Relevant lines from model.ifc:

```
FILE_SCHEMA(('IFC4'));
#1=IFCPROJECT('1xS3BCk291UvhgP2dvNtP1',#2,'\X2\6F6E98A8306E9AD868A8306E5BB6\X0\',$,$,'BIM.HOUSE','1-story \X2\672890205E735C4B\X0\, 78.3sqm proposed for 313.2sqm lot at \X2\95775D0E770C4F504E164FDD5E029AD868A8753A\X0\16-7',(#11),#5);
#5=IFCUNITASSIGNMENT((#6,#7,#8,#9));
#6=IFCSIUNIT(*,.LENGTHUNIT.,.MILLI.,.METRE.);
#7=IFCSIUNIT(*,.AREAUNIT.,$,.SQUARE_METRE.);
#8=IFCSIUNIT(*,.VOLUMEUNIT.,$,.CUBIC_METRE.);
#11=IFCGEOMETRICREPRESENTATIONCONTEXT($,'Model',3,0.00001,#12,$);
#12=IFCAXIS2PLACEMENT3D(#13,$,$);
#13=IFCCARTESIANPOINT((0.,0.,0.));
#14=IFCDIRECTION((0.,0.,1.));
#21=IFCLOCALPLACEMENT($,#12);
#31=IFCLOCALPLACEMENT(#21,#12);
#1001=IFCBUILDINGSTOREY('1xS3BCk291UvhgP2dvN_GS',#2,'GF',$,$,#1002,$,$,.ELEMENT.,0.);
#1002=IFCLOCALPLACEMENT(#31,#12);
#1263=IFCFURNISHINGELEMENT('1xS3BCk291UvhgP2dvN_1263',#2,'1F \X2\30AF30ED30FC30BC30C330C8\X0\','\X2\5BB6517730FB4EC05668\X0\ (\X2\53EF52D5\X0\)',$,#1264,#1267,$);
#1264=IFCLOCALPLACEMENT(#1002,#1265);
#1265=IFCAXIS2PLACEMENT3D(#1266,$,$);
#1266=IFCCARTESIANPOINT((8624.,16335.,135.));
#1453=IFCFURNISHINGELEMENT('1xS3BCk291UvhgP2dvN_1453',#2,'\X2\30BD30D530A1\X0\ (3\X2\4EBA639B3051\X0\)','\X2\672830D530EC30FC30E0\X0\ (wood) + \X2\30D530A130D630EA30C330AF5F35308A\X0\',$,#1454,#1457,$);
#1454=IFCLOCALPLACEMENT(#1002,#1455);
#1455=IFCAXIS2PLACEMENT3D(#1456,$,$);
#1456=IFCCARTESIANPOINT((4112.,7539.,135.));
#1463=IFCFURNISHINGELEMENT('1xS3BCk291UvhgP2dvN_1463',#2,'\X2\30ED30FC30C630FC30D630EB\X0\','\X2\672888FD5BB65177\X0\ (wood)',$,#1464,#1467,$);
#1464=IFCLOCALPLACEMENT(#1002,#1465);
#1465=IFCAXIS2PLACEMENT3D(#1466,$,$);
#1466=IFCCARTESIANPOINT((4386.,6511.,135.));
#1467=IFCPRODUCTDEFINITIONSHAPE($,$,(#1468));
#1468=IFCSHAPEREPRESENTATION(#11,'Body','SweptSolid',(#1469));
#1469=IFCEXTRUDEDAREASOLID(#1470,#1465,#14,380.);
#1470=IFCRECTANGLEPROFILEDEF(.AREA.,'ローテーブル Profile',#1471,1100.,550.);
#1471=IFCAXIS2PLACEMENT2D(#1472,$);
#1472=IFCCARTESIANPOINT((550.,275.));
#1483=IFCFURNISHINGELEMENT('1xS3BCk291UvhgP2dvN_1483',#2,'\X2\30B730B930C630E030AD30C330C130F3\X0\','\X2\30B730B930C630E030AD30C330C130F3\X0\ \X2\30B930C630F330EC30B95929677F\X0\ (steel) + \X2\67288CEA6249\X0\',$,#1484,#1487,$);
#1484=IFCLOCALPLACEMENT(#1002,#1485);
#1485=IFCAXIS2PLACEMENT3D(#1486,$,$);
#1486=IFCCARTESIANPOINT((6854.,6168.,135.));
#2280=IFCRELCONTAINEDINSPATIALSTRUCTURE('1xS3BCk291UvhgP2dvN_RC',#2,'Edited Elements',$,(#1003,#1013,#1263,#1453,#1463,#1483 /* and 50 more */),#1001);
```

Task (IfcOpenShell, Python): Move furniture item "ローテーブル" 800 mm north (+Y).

```python
import ifcopenshell
import ifcopenshell.api.geometry
import ifcopenshell.util.placement
import ifcopenshell.util.unit

model = ifcopenshell.open("model.ifc")
unit_scale = ifcopenshell.util.unit.calculate_unit_scale(model)

item = model.by_guid("1xS3BCk291UvhgP2dvN_1463")
matrix = ifcopenshell.util.placement.get_local_placement(item.ObjectPlacement)
matrix[1, 3] += 0.8 / unit_scale
ifcopenshell.api.geometry.edit_object_placement(model, product=item, matrix=matrix, is_si=False)

print(ifcopenshell.util.placement.get_local_placement(item.ObjectPlacement).round(3) + 0.0)

model.write("model_updated.ifc")
```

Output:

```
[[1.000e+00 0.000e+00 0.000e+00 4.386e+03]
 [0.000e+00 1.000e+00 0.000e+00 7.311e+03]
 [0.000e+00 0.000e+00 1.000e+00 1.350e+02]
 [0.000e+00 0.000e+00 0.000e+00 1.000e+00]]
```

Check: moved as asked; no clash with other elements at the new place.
